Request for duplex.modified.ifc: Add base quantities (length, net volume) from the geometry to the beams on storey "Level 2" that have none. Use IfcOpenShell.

First a look at what the model holds.

```python
import ifcopenshell
import ifcopenshell.util.element
import ifcopenshell.util.unit

model = ifcopenshell.open("duplex.modified.ifc")
print(model.schema)
for unit_type in ("LENGTHUNIT", "AREAUNIT", "VOLUMEUNIT"):
    print(unit_type, ifcopenshell.util.unit.calculate_unit_scale(model, unit_type))
storey = next(s for s in model.by_type("IfcBuildingStorey") if s.Name == "Level 2")
beams = [e for e in ifcopenshell.util.element.get_decomposition(storey) if e.is_a("IfcBeam")]
for e in sorted(beams, key=lambda e: e.id()):
    print(e.id(), e.is_a(), e.Name, list(ifcopenshell.util.element.get_psets(e, qtos_only=True)), sep=" | ")
```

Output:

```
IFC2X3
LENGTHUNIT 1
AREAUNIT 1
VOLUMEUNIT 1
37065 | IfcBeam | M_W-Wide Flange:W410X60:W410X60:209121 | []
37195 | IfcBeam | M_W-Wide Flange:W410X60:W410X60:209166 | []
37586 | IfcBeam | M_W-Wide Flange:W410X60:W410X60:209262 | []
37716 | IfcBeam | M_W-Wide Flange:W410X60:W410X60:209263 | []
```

```python
import ifcopenshell
import ifcopenshell.api.pset
import ifcopenshell.geom
import ifcopenshell.util.element
import ifcopenshell.util.shape
import ifcopenshell.util.unit

model = ifcopenshell.open("duplex.modified.ifc")
unit_scale = ifcopenshell.util.unit.calculate_unit_scale(model)
volume_scale = ifcopenshell.util.unit.calculate_unit_scale(model, "VOLUMEUNIT")
settings = ifcopenshell.geom.settings()

storey = next(s for s in model.by_type("IfcBuildingStorey") if s.Name == "Level 2")
beams = [e for e in ifcopenshell.util.element.get_decomposition(storey) if e.is_a("IfcBeam")]

for e in sorted(beams, key=lambda e: e.id()):
    if ifcopenshell.util.element.get_psets(e, qtos_only=True, should_inherit=False):
        continue
    # Geometry comes back in metres, in the element's own axes.
    shape = ifcopenshell.geom.create_shape(settings, e)
    values = {
        "Length": ifcopenshell.util.shape.get_max_xyz(shape.geometry) / unit_scale,
        "NetVolume": ifcopenshell.util.shape.get_volume(shape.geometry) / volume_scale,
    }
    qto = ifcopenshell.api.pset.add_qto(model, product=e, name="BaseQuantities")
    ifcopenshell.api.pset.edit_qto(model, qto=qto, properties=values)
    print(e.id(), {k: round(v, 3) for k, v in values.items()})

model.write("duplex.modified_v2.ifc")
```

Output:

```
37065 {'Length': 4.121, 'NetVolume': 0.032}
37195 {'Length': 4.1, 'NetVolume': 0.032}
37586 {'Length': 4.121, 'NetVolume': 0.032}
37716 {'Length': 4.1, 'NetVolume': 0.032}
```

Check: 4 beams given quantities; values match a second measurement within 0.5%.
